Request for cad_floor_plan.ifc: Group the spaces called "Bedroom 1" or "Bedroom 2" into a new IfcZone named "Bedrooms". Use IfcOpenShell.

First a look at what the model holds.

```python
import ifcopenshell

model = ifcopenshell.open("cad_floor_plan.ifc")
print(model.schema)
seen = {}
for space in model.by_type("IfcSpace"):
    seen[space.LongName] = seen.get(space.LongName, 0) + 1
for name, count in sorted(seen.items(), key=str):
    print(count, "x", name)
print("zones:", [z.Name for z in model.by_type("IfcZone")][:20])
```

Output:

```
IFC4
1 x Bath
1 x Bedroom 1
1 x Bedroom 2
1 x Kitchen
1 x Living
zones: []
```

```python
import ifcopenshell
import ifcopenshell.api.group
import ifcopenshell.api.root

model = ifcopenshell.open("cad_floor_plan.ifc")

names = {"Bedroom 1", "Bedroom 2"}
spaces = [s for s in model.by_type("IfcSpace") if s.LongName in names]

zone = ifcopenshell.api.root.create_entity(model, ifc_class="IfcZone", name="Bedrooms")
ifcopenshell.api.group.assign_group(model, products=spaces, group=zone)
print(len(spaces), "spaces in", zone.Name)

model.write("cad_floor_plan_v2.ifc")
```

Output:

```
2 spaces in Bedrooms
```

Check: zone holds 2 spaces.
